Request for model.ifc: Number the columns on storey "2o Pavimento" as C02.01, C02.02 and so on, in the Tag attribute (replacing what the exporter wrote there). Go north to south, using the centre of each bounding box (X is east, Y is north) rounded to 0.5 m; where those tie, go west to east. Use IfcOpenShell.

First a look at what the model holds.

```python
import ifcopenshell
import ifcopenshell.util.element
import ifcopenshell.util.placement

model = ifcopenshell.open("model.ifc")
print(model.schema)
storey = next(s for s in model.by_type("IfcBuildingStorey") if s.Name == "2o Pavimento")
columns = [e for e in ifcopenshell.util.element.get_decomposition(storey) if e.is_a("IfcColumn")]
for e in sorted(columns, key=lambda e: e.id()):
    origin = ifcopenshell.util.placement.get_local_placement(e.ObjectPlacement)[:3, 3]
    print(e.id(), e.Tag, e.Name, origin.round(2) + 0.0, sep=" | ")
```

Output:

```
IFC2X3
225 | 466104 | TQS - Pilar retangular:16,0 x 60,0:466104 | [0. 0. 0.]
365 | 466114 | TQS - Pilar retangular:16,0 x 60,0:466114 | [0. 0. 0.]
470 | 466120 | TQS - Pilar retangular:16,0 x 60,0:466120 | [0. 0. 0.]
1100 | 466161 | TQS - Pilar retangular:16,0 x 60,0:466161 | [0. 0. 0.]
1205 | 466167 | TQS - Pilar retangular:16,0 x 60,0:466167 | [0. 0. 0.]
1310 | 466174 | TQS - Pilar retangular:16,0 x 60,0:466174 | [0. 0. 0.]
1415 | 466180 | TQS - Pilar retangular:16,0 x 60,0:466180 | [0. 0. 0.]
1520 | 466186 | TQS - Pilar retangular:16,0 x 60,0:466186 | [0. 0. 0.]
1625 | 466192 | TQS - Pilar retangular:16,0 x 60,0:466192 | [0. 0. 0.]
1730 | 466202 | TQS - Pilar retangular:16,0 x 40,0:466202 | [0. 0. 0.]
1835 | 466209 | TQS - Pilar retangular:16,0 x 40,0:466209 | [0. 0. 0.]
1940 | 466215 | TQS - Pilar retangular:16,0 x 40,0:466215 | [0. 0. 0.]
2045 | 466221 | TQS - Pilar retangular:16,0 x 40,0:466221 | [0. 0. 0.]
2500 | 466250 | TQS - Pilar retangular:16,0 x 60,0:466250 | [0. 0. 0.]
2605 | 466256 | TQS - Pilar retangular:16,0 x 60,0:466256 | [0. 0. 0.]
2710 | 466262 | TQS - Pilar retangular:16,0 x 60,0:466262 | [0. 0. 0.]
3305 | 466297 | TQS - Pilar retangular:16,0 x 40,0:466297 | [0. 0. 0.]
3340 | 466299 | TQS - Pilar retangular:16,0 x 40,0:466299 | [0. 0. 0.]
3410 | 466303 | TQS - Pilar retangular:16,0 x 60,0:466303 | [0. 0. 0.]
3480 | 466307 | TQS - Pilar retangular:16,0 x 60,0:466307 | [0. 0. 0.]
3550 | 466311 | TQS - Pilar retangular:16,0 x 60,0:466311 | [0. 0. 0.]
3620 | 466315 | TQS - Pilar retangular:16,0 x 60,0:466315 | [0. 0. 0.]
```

```python
import ifcopenshell
import ifcopenshell.geom
import ifcopenshell.util.element
import ifcopenshell.util.shape

model = ifcopenshell.open("model.ifc")
settings = ifcopenshell.geom.settings()
settings.set("use-world-coords", True)


def centre(element):
    shape = ifcopenshell.geom.create_shape(settings, element)
    return ifcopenshell.util.shape.get_bbox_centroid(shape.geometry)


storey = next(s for s in model.by_type("IfcBuildingStorey") if s.Name == "2o Pavimento")
columns = [e for e in ifcopenshell.util.element.get_decomposition(storey) if e.is_a("IfcColumn")]

# Insertion points can sit at a corner or the storey origin, so sort by the geometry (in metres).
centres = {e: centre(e) for e in columns}
columns.sort(key=lambda e: (-round(centres[e][1] / 0.5), centres[e][0]))

for i, e in enumerate(columns, start=1):
    number = f"C02.{i:02d}"
    e.Tag = number
    print(e.id(), number)

model.write("model_rev.ifc")
```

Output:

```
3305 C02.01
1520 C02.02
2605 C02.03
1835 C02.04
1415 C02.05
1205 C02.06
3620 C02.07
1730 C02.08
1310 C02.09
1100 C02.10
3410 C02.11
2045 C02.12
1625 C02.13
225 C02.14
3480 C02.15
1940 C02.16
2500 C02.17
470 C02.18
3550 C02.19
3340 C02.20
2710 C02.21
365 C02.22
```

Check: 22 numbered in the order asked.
